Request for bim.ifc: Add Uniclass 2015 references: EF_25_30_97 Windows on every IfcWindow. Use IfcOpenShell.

First a look at what the model holds.

```python
import ifcopenshell

model = ifcopenshell.open("bim.ifc")
print(model.schema)
print("classifications:", [c.Name for c in model.by_type("IfcClassification")])
for ifc_class in ("IfcDoor", "IfcRoof", "IfcStair", "IfcWall", "IfcWindow"):
    print(ifc_class, len(model.by_type(ifc_class)))
```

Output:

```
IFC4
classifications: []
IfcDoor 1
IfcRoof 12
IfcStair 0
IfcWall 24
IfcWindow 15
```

```python
import ifcopenshell
import ifcopenshell.api.classification

model = ifcopenshell.open("bim.ifc")

system = ifcopenshell.api.classification.add_classification(model, classification="Uniclass 2015")

codes = {
    "IfcWindow": ("EF_25_30_97", "Windows"),
}
for ifc_class, (code, name) in codes.items():
    products = model.by_type(ifc_class)
    ifcopenshell.api.classification.add_reference(
        model, products=products, classification=system, identification=code, name=name
    )
    print(code, len(products))

model.write("bim_v2.ifc")
```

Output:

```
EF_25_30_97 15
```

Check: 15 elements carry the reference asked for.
